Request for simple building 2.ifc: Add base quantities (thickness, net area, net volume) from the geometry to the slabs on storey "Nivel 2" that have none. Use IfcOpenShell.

First a look at what the model holds.

```python
import ifcopenshell
import ifcopenshell.util.element
import ifcopenshell.util.unit

model = ifcopenshell.open("simple building 2.ifc")
print(model.schema)
for unit_type in ("LENGTHUNIT", "AREAUNIT", "VOLUMEUNIT"):
    print(unit_type, ifcopenshell.util.unit.calculate_unit_scale(model, unit_type))
storey = next(s for s in model.by_type("IfcBuildingStorey") if s.Name == "Nivel 2")
slabs = [e for e in ifcopenshell.util.element.get_decomposition(storey) if e.is_a("IfcSlab")]
for e in sorted(slabs, key=lambda e: e.id()):
    print(e.id(), e.is_a(), e.Name, list(ifcopenshell.util.element.get_psets(e, qtos_only=True)), sep=" | ")
```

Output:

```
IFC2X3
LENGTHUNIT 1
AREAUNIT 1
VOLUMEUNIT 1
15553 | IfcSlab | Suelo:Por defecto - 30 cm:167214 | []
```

```python
import ifcopenshell
import ifcopenshell.api.pset
import ifcopenshell.geom
import ifcopenshell.util.element
import ifcopenshell.util.shape
import ifcopenshell.util.unit

model = ifcopenshell.open("simple building 2.ifc")
unit_scale = ifcopenshell.util.unit.calculate_unit_scale(model)
area_scale = ifcopenshell.util.unit.calculate_unit_scale(model, "AREAUNIT")
volume_scale = ifcopenshell.util.unit.calculate_unit_scale(model, "VOLUMEUNIT")
settings = ifcopenshell.geom.settings()

storey = next(s for s in model.by_type("IfcBuildingStorey") if s.Name == "Nivel 2")
slabs = [e for e in ifcopenshell.util.element.get_decomposition(storey) if e.is_a("IfcSlab")]

for e in sorted(slabs, key=lambda e: e.id()):
    if ifcopenshell.util.element.get_psets(e, qtos_only=True, should_inherit=False):
        continue
    # Geometry comes back in metres, in the element's own axes.
    shape = ifcopenshell.geom.create_shape(settings, e)
    values = {
        "Width": ifcopenshell.util.shape.get_z(shape.geometry) / unit_scale,
        "NetArea": ifcopenshell.util.shape.get_footprint_area(shape.geometry) / area_scale,
        "NetVolume": ifcopenshell.util.shape.get_volume(shape.geometry) / volume_scale,
    }
    qto = ifcopenshell.api.pset.add_qto(model, product=e, name="BaseQuantities")
    ifcopenshell.api.pset.edit_qto(model, qto=qto, properties=values)
    print(e.id(), {k: round(v, 3) for k, v in values.items()})

model.write("simple building 2_edited.ifc")
```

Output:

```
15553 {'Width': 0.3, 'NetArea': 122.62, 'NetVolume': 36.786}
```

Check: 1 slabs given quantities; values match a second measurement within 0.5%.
